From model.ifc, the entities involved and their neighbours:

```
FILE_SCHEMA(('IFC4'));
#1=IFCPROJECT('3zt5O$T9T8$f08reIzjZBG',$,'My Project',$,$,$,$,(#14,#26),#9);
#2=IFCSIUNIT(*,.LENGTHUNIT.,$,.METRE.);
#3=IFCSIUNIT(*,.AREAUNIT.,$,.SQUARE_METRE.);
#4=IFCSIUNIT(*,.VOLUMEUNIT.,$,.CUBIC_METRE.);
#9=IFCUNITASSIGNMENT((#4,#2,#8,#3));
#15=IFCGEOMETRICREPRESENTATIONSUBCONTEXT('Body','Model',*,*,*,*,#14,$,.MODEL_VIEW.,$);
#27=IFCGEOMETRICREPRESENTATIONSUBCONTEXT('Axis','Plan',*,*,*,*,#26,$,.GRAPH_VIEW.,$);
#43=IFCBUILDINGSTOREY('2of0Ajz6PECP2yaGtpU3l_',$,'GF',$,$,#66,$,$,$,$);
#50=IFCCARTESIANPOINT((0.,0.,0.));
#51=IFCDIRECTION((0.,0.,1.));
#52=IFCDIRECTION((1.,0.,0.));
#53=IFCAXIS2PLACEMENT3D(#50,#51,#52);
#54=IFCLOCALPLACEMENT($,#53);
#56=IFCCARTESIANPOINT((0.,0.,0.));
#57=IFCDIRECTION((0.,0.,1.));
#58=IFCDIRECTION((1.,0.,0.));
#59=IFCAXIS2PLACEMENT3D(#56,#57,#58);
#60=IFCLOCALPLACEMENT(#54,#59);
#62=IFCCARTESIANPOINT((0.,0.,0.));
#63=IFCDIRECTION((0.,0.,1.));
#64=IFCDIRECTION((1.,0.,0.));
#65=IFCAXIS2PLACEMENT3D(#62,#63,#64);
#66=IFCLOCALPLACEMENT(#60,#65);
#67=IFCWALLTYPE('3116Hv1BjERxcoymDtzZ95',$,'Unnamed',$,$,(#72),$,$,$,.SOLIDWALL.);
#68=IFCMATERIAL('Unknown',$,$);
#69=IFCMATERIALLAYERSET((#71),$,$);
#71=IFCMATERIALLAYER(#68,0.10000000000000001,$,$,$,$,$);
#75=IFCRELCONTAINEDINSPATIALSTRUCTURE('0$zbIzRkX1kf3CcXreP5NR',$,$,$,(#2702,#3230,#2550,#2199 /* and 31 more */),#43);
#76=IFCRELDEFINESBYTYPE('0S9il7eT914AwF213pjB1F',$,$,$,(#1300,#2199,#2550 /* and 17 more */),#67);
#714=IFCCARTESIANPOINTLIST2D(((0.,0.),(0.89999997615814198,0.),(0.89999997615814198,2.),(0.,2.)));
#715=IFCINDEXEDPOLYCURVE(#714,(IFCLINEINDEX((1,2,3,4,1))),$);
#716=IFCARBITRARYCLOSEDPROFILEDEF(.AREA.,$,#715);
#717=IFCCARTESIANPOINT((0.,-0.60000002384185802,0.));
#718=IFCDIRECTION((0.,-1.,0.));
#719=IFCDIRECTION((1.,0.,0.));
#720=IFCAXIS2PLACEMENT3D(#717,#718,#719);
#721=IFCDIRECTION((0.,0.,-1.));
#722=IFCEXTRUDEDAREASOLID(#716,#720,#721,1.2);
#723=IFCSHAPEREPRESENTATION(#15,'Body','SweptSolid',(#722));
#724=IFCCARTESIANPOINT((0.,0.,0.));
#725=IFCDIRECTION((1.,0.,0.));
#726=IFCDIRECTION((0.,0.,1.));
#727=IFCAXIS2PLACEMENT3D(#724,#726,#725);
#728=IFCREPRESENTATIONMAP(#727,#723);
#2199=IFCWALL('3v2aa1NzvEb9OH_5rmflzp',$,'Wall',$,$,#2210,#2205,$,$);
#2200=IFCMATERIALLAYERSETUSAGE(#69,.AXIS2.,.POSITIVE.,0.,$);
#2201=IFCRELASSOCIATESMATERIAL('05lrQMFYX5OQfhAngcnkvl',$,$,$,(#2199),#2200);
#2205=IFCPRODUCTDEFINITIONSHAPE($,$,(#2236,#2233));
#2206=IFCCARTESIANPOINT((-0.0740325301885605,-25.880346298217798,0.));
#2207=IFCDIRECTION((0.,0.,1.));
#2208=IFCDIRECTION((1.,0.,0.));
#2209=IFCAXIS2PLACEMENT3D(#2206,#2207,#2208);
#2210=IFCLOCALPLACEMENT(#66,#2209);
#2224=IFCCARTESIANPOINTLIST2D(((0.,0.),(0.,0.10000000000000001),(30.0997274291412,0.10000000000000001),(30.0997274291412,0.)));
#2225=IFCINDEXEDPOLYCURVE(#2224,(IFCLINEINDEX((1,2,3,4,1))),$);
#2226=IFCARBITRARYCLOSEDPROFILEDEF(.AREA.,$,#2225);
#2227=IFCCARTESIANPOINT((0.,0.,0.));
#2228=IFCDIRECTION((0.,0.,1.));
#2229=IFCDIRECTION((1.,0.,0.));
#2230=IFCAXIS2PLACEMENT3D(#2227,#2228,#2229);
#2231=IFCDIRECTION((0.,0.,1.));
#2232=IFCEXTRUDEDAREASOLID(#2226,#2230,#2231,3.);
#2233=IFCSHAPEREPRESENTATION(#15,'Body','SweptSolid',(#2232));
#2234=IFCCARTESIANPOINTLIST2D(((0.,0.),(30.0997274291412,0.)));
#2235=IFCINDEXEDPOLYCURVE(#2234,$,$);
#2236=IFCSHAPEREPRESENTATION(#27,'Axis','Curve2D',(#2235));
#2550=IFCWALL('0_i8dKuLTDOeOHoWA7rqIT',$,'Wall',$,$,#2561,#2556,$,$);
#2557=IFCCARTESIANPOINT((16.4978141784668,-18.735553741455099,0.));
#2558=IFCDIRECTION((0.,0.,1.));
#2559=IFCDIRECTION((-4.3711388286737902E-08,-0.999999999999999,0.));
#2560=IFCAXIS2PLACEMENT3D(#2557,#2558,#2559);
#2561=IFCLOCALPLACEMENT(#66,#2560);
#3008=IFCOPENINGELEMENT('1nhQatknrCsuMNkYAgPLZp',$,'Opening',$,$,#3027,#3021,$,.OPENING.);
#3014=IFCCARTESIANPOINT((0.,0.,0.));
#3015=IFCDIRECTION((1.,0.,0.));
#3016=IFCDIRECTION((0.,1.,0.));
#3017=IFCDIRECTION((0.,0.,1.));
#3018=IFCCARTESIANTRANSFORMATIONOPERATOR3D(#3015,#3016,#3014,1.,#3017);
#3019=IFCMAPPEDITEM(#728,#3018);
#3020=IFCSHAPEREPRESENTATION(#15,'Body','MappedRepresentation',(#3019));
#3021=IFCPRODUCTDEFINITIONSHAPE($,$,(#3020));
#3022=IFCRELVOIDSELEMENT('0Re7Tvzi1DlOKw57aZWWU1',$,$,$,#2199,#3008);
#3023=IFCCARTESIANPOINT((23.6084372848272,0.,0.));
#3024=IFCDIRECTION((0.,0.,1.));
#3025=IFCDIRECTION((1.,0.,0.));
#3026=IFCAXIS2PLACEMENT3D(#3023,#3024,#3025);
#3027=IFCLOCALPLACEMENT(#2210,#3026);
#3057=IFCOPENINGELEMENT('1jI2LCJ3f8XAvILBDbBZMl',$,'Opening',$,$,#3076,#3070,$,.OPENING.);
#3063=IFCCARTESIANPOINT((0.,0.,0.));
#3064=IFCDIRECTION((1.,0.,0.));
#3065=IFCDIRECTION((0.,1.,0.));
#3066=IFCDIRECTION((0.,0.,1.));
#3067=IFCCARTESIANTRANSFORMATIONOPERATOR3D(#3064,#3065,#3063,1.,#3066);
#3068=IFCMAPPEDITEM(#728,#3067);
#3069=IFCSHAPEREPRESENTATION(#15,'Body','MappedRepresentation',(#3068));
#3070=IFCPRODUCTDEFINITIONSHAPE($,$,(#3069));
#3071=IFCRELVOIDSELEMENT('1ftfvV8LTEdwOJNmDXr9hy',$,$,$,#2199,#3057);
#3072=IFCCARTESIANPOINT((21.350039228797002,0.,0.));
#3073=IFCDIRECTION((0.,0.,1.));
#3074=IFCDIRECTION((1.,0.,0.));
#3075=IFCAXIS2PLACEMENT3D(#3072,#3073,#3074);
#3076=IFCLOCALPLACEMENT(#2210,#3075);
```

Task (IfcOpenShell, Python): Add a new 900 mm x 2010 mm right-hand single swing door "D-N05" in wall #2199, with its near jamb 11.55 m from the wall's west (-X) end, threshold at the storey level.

```python
import numpy as np
import ifcopenshell
import ifcopenshell.api.feature
import ifcopenshell.api.geometry
import ifcopenshell.api.root
import ifcopenshell.api.spatial
import ifcopenshell.geom
import ifcopenshell.util.element
import ifcopenshell.util.placement
import ifcopenshell.util.representation
import ifcopenshell.util.shape
import ifcopenshell.util.unit

model = ifcopenshell.open("model.ifc")
unit_scale = ifcopenshell.util.unit.calculate_unit_scale(model)
settings = ifcopenshell.geom.settings()


def volume(element):
    """Net volume in cubic metres, openings subtracted."""
    shape = ifcopenshell.geom.create_shape(settings, element)
    return ifcopenshell.util.shape.get_volume(shape.geometry)


wall = model.by_guid("3v2aa1NzvEb9OH_5rmflzp")
storey = ifcopenshell.util.element.get_container(wall, ifc_class="IfcBuildingStorey")
context = ifcopenshell.util.representation.get_context(model, "Model", "Body", "MODEL_VIEW")
before = volume(wall)

width, height, from_end, sill = 0.9, 2.01, 11.55, 0.0  # metres

# The wall runs along its own X axis, and the end named is its -X end.
wall_shape = ifcopenshell.geom.create_shape(settings, wall)
x, y, z = ifcopenshell.util.shape.get_vertices(wall_shape.geometry).T
start = x.min() + from_end
face, thickness = float(y.min()), float(y.max() - y.min())
wall_matrix = ifcopenshell.util.placement.get_local_placement(wall.ObjectPlacement)
level = ifcopenshell.util.placement.get_local_placement(storey.ObjectPlacement)[2, 3]


def in_wall(x, y):
    """Placement at x, y metres in the wall's axes, at sill height."""
    matrix = wall_matrix.copy()
    matrix[:, 3] = wall_matrix @ np.array([x / unit_scale, y / unit_scale, 0.0, 1.0])
    matrix[2, 3] = level + sill / unit_scale
    return matrix


# Opening: a box that overshoots both wall faces by 50 mm.
opening = ifcopenshell.api.root.create_entity(model, ifc_class="IfcOpeningElement", predefined_type="OPENING")
box = ifcopenshell.api.geometry.add_wall_representation(
    model, context=context, length=width, height=height, thickness=thickness + 0.1
)
ifcopenshell.api.geometry.assign_representation(model, product=opening, representation=box)
ifcopenshell.api.geometry.edit_object_placement(model, product=opening, matrix=in_wall(start, face - 0.05), is_si=False)
ifcopenshell.api.feature.add_feature(model, feature=opening, element=wall)

door = ifcopenshell.api.root.create_entity(model, ifc_class="IfcDoor", name="D-N05", predefined_type="DOOR")
door.OverallWidth, door.OverallHeight = width / unit_scale, height / unit_scale
door.OperationType = "SINGLE_SWING_RIGHT"
body = ifcopenshell.api.geometry.add_door_representation(
    model,
    context=context,
    overall_width=door.OverallWidth,
    overall_height=door.OverallHeight,
    operation_type="SINGLE_SWING_RIGHT",
    lining_properties={"LiningDepth": thickness / unit_scale, "ThresholdDepth": thickness / unit_scale},
)
ifcopenshell.api.geometry.assign_representation(model, product=door, representation=body)
ifcopenshell.api.spatial.assign_container(model, products=[door], relating_structure=storey)
ifcopenshell.api.feature.add_filling(model, opening=opening, element=door)

# The lining spans the wall, so the door starts at the wall face.
ifcopenshell.api.geometry.edit_object_placement(model, product=door, matrix=in_wall(start, face), is_si=False)

after = volume(wall)

print(f"wall volume {before:.3f} -> {after:.3f} m3")

model.write("model-out.ifc")
```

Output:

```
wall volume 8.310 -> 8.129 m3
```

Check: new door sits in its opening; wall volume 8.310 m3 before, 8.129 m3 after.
